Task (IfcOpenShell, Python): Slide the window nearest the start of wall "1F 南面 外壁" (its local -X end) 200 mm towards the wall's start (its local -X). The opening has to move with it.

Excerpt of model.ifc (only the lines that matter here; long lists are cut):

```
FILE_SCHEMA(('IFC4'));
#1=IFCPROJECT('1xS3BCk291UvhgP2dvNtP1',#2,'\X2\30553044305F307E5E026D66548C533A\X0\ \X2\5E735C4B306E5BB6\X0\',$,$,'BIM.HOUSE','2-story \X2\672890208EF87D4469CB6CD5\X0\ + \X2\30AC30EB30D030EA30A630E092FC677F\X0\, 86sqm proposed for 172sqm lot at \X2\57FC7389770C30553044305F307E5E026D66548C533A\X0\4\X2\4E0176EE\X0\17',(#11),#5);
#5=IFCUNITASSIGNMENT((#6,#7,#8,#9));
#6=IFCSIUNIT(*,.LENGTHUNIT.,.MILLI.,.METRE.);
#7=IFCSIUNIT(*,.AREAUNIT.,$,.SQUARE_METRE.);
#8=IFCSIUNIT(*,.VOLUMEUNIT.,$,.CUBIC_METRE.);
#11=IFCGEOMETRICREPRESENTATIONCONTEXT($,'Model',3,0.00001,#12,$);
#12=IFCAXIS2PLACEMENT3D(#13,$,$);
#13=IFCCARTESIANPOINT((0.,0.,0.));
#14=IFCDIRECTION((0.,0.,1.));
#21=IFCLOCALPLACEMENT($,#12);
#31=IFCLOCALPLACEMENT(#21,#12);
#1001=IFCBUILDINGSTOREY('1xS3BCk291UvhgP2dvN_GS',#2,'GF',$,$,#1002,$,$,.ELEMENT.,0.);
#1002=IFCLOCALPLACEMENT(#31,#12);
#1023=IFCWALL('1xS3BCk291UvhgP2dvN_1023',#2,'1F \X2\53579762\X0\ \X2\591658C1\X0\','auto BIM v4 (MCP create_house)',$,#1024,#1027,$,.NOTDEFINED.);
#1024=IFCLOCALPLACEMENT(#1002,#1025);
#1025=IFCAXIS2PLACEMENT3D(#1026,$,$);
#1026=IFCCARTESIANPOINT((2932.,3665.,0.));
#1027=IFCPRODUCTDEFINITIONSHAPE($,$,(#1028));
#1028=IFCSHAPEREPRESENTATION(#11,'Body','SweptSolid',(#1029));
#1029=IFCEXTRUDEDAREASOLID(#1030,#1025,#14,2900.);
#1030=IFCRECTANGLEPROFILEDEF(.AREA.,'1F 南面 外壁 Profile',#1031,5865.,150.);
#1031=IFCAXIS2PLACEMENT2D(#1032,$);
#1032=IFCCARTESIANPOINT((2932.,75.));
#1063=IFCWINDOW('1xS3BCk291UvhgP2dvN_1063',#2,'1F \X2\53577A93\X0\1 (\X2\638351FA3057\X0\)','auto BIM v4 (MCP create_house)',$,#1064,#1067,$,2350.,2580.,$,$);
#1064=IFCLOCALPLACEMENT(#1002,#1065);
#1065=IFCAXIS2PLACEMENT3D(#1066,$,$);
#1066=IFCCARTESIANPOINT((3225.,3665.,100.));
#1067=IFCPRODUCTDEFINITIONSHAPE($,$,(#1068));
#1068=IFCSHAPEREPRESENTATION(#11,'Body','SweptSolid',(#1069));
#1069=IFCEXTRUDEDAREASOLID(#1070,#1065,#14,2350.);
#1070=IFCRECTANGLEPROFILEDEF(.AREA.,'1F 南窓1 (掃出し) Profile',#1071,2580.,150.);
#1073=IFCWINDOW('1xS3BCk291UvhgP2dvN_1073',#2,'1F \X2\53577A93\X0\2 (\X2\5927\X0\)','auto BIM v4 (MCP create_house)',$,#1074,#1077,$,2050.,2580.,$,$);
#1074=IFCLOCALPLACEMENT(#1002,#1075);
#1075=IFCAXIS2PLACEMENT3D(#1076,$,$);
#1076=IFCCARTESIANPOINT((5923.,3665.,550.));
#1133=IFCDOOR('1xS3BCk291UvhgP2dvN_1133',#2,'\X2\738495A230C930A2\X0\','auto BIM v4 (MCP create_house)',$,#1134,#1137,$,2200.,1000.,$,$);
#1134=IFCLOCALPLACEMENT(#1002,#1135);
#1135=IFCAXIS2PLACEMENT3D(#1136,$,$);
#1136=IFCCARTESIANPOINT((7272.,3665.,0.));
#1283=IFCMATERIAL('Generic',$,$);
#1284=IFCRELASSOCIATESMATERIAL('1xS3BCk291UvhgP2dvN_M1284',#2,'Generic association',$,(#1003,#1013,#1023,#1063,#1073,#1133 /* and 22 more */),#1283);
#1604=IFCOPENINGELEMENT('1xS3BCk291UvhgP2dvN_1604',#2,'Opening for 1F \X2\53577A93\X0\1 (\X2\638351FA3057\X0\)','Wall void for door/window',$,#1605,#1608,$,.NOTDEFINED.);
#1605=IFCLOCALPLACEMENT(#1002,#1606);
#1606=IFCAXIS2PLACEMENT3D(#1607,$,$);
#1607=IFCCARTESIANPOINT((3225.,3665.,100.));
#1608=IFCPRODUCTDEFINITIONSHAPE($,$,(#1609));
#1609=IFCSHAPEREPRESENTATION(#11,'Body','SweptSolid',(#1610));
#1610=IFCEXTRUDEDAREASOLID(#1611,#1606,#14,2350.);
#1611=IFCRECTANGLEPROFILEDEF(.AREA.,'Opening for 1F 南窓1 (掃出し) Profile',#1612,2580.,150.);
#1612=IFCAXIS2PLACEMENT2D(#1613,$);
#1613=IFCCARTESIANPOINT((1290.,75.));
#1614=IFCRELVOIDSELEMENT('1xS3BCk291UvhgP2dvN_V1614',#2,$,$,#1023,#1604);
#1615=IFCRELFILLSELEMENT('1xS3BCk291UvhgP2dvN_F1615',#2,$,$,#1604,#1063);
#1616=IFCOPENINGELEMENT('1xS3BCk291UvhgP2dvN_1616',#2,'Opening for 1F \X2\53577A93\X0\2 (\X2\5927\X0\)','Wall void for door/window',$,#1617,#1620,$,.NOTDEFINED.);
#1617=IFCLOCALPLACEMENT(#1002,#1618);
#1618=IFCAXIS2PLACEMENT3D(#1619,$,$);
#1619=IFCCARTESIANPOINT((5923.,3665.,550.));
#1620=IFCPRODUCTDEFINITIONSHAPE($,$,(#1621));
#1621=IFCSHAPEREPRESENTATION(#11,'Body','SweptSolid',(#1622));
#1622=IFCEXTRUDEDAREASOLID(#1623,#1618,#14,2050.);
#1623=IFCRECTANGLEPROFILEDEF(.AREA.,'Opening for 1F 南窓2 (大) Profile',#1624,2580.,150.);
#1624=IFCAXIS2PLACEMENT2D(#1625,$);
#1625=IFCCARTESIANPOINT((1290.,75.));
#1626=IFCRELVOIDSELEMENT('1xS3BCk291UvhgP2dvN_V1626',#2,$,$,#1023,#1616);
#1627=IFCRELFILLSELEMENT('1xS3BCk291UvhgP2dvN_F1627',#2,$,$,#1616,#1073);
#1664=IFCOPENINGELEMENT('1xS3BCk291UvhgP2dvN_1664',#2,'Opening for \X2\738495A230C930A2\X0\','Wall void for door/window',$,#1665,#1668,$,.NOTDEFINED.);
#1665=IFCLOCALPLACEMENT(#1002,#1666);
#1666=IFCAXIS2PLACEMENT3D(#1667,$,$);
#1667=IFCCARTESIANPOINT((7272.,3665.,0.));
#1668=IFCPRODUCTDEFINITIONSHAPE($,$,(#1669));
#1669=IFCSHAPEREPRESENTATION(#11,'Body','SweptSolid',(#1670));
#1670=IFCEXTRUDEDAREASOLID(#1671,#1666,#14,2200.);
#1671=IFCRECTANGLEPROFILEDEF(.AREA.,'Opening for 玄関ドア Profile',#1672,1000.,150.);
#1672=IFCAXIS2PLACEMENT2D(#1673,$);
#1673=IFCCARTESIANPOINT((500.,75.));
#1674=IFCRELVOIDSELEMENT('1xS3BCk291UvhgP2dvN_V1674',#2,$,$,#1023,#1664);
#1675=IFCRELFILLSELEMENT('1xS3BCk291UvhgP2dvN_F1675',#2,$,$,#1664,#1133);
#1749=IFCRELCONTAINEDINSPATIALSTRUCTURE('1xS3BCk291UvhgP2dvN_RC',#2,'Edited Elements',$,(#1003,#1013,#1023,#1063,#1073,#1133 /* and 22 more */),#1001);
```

```python
import ifcopenshell
import ifcopenshell.api.geometry
import ifcopenshell.util.placement
import ifcopenshell.util.unit

model = ifcopenshell.open("model.ifc")
unit_scale = ifcopenshell.util.unit.calculate_unit_scale(model)

window = model.by_guid("1xS3BCk291UvhgP2dvN_1063")
opening = window.FillsVoids[0].RelatingOpeningElement
wall = opening.VoidsElements[0].RelatingBuildingElement

wall_matrix = ifcopenshell.util.placement.get_local_placement(wall.ObjectPlacement)
shift = wall_matrix[:3, 0] * -0.2 / unit_scale
before = ifcopenshell.util.placement.get_local_placement(window.ObjectPlacement)[:3, 3].copy()

# The window is not placed relative to its opening, so move both.
for product in (opening, window):
    matrix = ifcopenshell.util.placement.get_local_placement(product.ObjectPlacement)
    matrix[:3, 3] += shift
    ifcopenshell.api.geometry.edit_object_placement(model, product=product, matrix=matrix, is_si=False)

after = ifcopenshell.util.placement.get_local_placement(window.ObjectPlacement)[:3, 3]
print("window moved by", (after - before).round(3) + 0.0)

model.write("model-out.ifc")
```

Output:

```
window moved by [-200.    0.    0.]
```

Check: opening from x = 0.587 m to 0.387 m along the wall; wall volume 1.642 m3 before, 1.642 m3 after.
